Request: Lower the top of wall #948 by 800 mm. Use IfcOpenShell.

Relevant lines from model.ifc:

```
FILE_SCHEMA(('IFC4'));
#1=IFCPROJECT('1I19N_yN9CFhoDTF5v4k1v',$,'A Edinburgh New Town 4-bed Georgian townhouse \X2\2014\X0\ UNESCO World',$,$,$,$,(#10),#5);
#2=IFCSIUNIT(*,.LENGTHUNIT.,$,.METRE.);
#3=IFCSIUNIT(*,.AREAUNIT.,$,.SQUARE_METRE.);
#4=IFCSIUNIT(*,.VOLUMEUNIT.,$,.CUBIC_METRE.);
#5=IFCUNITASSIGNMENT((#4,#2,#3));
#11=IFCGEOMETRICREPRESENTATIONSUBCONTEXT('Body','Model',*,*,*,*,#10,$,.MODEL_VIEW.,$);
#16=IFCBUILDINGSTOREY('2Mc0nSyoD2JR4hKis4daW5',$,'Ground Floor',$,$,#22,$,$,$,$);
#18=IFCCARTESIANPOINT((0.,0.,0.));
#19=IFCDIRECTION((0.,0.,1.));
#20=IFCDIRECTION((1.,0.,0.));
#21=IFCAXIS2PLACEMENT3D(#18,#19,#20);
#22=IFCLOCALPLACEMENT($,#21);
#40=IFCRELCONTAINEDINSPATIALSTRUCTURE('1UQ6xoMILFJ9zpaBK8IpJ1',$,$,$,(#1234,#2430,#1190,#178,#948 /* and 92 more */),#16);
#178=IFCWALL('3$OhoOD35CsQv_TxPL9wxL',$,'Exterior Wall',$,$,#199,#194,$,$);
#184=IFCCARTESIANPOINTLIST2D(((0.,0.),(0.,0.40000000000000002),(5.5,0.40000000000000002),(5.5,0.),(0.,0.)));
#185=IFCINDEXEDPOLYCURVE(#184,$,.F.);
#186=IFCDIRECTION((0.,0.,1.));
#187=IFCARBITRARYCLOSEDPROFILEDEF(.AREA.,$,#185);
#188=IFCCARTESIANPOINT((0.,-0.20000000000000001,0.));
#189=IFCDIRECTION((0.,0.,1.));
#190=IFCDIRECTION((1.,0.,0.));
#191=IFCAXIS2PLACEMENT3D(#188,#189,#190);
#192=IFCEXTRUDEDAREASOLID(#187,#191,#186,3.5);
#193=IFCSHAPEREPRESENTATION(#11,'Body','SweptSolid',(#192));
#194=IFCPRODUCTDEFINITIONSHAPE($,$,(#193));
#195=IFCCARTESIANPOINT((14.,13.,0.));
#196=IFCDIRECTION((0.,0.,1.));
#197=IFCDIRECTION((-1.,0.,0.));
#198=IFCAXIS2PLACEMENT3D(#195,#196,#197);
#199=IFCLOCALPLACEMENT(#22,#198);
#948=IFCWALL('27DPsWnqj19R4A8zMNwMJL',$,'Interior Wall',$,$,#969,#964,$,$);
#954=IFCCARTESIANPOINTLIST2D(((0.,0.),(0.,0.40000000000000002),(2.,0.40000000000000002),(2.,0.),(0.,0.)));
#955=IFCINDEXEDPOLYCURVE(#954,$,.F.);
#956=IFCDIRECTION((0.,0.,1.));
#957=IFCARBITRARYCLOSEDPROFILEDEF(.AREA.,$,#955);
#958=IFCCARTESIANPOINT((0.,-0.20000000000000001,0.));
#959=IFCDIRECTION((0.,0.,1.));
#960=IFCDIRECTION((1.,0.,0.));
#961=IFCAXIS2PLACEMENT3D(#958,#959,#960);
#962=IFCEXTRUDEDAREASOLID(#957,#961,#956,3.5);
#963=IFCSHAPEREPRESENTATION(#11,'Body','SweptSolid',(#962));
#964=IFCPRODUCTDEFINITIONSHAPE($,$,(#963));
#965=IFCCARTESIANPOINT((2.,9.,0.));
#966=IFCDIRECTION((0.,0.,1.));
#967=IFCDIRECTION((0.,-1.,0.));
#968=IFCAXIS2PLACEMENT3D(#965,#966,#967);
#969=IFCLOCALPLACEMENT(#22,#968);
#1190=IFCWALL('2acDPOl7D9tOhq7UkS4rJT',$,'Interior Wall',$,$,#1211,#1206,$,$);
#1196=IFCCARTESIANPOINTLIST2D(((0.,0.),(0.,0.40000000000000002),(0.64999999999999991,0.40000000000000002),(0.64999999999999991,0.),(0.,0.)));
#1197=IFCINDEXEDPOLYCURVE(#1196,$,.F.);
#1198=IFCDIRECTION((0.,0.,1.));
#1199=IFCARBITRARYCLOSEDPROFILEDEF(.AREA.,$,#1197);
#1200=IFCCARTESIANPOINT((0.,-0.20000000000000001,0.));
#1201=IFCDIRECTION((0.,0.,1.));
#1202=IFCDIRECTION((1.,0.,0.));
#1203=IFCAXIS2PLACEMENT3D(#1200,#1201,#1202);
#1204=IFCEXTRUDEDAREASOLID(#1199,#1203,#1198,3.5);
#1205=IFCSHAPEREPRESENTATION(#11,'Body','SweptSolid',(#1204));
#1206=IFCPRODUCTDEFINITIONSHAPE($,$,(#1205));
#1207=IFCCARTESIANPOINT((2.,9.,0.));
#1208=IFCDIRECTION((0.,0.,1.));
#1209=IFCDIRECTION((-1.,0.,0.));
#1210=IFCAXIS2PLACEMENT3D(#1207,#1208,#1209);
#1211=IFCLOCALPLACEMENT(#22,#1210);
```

```python
import ifcopenshell
import ifcopenshell.geom
import ifcopenshell.util.representation
import ifcopenshell.util.shape

model = ifcopenshell.open("model.ifc")
settings = ifcopenshell.geom.settings()


def volume(element):
    """Net volume in cubic metres, openings subtracted."""
    shape = ifcopenshell.geom.create_shape(settings, element)
    return ifcopenshell.util.shape.get_volume(shape.geometry)


wall = model.by_id(948)
before = volume(wall)

body = ifcopenshell.util.representation.get_representation(wall, "Model", "Body")
solid = body.Items[0]
old_height = solid.Depth
solid.Depth -= 0.8
after = volume(wall)

print(f"height {old_height:g} -> {solid.Depth:g}, volume {before:.3f} -> {after:.3f} m3")

model.write("model_v2.ifc")
```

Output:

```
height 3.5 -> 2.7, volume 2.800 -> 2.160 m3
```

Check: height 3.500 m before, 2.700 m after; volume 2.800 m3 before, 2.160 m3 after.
